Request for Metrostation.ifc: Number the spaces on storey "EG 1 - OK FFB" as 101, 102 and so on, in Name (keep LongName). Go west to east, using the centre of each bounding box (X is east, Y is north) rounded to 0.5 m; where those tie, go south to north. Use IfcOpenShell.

First a look at what the model holds.

```python
import ifcopenshell
import ifcopenshell.util.element
import ifcopenshell.util.placement

model = ifcopenshell.open("Metrostation.ifc")
print(model.schema)
storey = next(s for s in model.by_type("IfcBuildingStorey") if s.Name == "EG 1 - OK FFB")
spaces = [e for e in ifcopenshell.util.element.get_decomposition(storey) if e.is_a("IfcSpace")]
for e in sorted(spaces, key=lambda e: e.id()):
    origin = ifcopenshell.util.placement.get_local_placement(e.ObjectPlacement)[:3, 3]
    print(e.id(), e.Name, e.LongName, origin.round(2) + 0.0, sep=" | ")
```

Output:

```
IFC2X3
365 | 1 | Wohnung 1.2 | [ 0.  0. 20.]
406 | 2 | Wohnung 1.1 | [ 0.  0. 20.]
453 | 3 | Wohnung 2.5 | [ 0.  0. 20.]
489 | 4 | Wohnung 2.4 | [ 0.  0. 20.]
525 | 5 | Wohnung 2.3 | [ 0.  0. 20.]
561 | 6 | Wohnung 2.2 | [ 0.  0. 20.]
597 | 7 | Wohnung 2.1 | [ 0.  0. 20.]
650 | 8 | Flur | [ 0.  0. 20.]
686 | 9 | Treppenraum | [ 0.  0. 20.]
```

```python
import ifcopenshell
import ifcopenshell.geom
import ifcopenshell.util.element
import ifcopenshell.util.shape

model = ifcopenshell.open("Metrostation.ifc")
settings = ifcopenshell.geom.settings()
settings.set("use-world-coords", True)


def centre(element):
    shape = ifcopenshell.geom.create_shape(settings, element)
    return ifcopenshell.util.shape.get_bbox_centroid(shape.geometry)


storey = next(s for s in model.by_type("IfcBuildingStorey") if s.Name == "EG 1 - OK FFB")
spaces = [e for e in ifcopenshell.util.element.get_decomposition(storey) if e.is_a("IfcSpace")]

# Insertion points can sit at a corner or the storey origin, so sort by the geometry (in metres).
centres = {e: centre(e) for e in spaces}
spaces.sort(key=lambda e: (round(centres[e][0] / 0.5), centres[e][1]))

for i, e in enumerate(spaces, start=1):
    number = f"1{i:02d}"
    e.Name = number
    print(e.id(), number)

model.write("Metrostation-out.ifc")
```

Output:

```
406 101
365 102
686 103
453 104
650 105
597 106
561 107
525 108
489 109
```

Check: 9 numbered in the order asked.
